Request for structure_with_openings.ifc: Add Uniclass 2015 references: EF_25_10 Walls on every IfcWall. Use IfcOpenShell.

First a look at what the model holds.

```python
import ifcopenshell

model = ifcopenshell.open("structure_with_openings.ifc")
print(model.schema)
print("classifications:", [c.Name for c in model.by_type("IfcClassification")])
for ifc_class in ("IfcDoor", "IfcRoof", "IfcStair", "IfcWall", "IfcWindow"):
    print(ifc_class, len(model.by_type(ifc_class)))
```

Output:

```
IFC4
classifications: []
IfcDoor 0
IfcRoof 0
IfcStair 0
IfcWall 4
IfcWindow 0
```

```python
import ifcopenshell
import ifcopenshell.api.classification

model = ifcopenshell.open("structure_with_openings.ifc")

system = ifcopenshell.api.classification.add_classification(model, classification="Uniclass 2015")

codes = {
    "IfcWall": ("EF_25_10", "Walls"),
}
for ifc_class, (code, name) in codes.items():
    products = model.by_type(ifc_class)
    ifcopenshell.api.classification.add_reference(
        model, products=products, classification=system, identification=code, name=name
    )
    print(code, len(products))

model.write("structure_with_openings_edited.ifc")
```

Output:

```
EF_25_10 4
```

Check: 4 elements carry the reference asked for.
